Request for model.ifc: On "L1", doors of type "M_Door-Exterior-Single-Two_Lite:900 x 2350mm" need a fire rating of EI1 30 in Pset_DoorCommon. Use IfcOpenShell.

First a look at what the model holds.

```python
import ifcopenshell
import ifcopenshell.util.element

model = ifcopenshell.open("model.ifc")
print(model.schema)
storey = next(s for s in model.by_type("IfcBuildingStorey") if s.Name == "L1")
doors = [e for e in ifcopenshell.util.element.get_decomposition(storey) if e.is_a("IfcDoor")]
seen = {}
for e in doors:
    element_type = ifcopenshell.util.element.get_type(e)
    key = (element_type.Name if element_type != e and element_type else None, ifcopenshell.util.element.get_pset(e, "Pset_DoorCommon", "FireRating"))
    seen[key] = seen.get(key, 0) + 1
for (name, value), count in sorted(seen.items(), key=str):
    print(count, "x", name, "|", value)
```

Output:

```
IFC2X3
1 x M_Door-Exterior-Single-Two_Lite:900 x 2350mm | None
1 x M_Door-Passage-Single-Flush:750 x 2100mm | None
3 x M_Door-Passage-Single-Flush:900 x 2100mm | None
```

```python
import ifcopenshell
import ifcopenshell.api.pset
import ifcopenshell.util.element

model = ifcopenshell.open("model.ifc")

storey = next(s for s in model.by_type("IfcBuildingStorey") if s.Name == "L1")
doors = [e for e in ifcopenshell.util.element.get_decomposition(storey) if e.is_a("IfcDoor")]

count = 0
for e in doors:
    element_type = ifcopenshell.util.element.get_type(e)
    if element_type in (None, e) or element_type.Name != "M_Door-Exterior-Single-Two_Lite:900 x 2350mm":
        continue
    # add_pset returns the element's existing set when there is one.
    pset = ifcopenshell.api.pset.add_pset(model, product=e, name="Pset_DoorCommon")
    ifcopenshell.api.pset.edit_pset(model, pset=pset, properties={"FireRating": "EI1 30"})
    count += 1

print(count, "doors updated")

model.write("model_updated.ifc")
```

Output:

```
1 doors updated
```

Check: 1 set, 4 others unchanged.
